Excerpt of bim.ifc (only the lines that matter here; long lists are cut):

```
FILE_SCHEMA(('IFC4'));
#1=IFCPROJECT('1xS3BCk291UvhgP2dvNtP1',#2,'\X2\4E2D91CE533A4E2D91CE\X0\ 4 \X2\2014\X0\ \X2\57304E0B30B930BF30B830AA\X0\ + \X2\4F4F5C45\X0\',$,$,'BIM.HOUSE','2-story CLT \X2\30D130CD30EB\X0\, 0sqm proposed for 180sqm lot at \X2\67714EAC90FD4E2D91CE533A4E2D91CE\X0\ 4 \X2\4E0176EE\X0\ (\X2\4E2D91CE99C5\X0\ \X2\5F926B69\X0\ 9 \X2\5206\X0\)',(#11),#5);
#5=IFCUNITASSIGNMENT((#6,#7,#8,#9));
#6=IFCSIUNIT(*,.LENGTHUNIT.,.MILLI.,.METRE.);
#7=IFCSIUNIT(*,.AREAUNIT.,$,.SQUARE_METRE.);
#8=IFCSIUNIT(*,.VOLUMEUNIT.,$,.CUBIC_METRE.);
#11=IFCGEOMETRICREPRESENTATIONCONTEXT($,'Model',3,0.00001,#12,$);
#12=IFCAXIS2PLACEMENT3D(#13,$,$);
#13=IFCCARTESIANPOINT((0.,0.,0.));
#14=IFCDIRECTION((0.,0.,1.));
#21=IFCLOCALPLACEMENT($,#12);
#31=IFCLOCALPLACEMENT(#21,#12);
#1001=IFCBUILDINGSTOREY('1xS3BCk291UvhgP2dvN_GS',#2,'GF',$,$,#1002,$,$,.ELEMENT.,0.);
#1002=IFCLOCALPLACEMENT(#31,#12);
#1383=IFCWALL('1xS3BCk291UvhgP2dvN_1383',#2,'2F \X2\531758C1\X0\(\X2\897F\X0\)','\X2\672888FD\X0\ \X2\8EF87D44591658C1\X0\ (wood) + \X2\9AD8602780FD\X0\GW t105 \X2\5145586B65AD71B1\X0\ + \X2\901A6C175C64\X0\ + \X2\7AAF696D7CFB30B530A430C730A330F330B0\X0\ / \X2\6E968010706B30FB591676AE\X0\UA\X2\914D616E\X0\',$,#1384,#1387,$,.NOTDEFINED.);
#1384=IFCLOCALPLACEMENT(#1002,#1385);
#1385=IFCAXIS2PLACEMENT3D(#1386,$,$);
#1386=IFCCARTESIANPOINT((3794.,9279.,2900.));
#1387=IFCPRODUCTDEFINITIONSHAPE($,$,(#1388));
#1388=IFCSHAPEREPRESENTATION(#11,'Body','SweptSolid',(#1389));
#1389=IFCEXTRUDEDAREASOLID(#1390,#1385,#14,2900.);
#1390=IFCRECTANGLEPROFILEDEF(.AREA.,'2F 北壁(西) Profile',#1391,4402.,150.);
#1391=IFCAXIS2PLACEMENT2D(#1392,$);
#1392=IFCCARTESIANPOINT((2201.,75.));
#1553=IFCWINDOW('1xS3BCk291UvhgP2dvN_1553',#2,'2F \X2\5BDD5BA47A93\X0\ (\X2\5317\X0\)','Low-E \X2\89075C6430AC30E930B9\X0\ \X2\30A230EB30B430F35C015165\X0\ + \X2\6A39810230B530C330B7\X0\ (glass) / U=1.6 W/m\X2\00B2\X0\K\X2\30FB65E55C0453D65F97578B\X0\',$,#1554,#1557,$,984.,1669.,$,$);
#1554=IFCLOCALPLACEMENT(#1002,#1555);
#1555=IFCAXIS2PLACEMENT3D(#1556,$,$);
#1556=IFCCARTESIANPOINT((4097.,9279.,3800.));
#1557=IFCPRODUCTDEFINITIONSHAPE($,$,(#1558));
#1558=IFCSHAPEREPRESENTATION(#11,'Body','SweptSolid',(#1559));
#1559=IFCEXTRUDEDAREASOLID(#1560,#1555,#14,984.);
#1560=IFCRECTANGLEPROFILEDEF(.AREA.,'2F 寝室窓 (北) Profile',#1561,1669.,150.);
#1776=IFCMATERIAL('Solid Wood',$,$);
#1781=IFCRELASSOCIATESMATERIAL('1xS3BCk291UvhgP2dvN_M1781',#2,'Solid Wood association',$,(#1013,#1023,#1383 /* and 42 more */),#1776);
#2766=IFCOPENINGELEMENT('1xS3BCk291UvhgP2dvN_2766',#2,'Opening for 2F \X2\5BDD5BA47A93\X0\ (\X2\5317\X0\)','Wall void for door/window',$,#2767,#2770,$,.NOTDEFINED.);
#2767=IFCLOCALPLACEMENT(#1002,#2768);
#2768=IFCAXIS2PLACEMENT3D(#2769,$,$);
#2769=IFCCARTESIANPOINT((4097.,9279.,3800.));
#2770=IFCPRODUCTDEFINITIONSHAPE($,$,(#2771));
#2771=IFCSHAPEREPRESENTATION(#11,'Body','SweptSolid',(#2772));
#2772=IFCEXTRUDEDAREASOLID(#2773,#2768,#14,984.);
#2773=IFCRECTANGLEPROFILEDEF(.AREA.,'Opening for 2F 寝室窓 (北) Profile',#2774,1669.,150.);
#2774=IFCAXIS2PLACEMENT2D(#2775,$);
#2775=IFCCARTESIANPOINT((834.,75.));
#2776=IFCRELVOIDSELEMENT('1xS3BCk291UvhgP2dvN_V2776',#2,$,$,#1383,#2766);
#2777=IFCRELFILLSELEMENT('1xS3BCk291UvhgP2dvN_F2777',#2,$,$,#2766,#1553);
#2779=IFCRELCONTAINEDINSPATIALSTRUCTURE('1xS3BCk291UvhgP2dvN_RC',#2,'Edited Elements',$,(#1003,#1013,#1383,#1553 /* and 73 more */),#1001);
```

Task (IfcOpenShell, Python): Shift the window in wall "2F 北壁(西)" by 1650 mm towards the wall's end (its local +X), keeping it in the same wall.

```python
import ifcopenshell
import ifcopenshell.api.geometry
import ifcopenshell.util.placement

model = ifcopenshell.open("bim.ifc")

window = model.by_guid("1xS3BCk291UvhgP2dvN_1553")
opening = window.FillsVoids[0].RelatingOpeningElement
wall = opening.VoidsElements[0].RelatingBuildingElement

wall_matrix = ifcopenshell.util.placement.get_local_placement(wall.ObjectPlacement)
shift = wall_matrix[:3, 0] * 1650.0
before = ifcopenshell.util.placement.get_local_placement(window.ObjectPlacement)[:3, 3].copy()

# The window is not placed relative to its opening, so move both.
for product in (opening, window):
    matrix = ifcopenshell.util.placement.get_local_placement(product.ObjectPlacement)
    matrix[:3, 3] += shift
    ifcopenshell.api.geometry.edit_object_placement(model, product=product, matrix=matrix, is_si=False)

after = ifcopenshell.util.placement.get_local_placement(window.ObjectPlacement)[:3, 3]
print("window moved by", (after - before).round(3) + 0.0)

model.write("bim_updated.ifc")
```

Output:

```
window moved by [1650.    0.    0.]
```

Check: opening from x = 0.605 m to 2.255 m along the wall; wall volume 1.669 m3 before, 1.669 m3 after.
